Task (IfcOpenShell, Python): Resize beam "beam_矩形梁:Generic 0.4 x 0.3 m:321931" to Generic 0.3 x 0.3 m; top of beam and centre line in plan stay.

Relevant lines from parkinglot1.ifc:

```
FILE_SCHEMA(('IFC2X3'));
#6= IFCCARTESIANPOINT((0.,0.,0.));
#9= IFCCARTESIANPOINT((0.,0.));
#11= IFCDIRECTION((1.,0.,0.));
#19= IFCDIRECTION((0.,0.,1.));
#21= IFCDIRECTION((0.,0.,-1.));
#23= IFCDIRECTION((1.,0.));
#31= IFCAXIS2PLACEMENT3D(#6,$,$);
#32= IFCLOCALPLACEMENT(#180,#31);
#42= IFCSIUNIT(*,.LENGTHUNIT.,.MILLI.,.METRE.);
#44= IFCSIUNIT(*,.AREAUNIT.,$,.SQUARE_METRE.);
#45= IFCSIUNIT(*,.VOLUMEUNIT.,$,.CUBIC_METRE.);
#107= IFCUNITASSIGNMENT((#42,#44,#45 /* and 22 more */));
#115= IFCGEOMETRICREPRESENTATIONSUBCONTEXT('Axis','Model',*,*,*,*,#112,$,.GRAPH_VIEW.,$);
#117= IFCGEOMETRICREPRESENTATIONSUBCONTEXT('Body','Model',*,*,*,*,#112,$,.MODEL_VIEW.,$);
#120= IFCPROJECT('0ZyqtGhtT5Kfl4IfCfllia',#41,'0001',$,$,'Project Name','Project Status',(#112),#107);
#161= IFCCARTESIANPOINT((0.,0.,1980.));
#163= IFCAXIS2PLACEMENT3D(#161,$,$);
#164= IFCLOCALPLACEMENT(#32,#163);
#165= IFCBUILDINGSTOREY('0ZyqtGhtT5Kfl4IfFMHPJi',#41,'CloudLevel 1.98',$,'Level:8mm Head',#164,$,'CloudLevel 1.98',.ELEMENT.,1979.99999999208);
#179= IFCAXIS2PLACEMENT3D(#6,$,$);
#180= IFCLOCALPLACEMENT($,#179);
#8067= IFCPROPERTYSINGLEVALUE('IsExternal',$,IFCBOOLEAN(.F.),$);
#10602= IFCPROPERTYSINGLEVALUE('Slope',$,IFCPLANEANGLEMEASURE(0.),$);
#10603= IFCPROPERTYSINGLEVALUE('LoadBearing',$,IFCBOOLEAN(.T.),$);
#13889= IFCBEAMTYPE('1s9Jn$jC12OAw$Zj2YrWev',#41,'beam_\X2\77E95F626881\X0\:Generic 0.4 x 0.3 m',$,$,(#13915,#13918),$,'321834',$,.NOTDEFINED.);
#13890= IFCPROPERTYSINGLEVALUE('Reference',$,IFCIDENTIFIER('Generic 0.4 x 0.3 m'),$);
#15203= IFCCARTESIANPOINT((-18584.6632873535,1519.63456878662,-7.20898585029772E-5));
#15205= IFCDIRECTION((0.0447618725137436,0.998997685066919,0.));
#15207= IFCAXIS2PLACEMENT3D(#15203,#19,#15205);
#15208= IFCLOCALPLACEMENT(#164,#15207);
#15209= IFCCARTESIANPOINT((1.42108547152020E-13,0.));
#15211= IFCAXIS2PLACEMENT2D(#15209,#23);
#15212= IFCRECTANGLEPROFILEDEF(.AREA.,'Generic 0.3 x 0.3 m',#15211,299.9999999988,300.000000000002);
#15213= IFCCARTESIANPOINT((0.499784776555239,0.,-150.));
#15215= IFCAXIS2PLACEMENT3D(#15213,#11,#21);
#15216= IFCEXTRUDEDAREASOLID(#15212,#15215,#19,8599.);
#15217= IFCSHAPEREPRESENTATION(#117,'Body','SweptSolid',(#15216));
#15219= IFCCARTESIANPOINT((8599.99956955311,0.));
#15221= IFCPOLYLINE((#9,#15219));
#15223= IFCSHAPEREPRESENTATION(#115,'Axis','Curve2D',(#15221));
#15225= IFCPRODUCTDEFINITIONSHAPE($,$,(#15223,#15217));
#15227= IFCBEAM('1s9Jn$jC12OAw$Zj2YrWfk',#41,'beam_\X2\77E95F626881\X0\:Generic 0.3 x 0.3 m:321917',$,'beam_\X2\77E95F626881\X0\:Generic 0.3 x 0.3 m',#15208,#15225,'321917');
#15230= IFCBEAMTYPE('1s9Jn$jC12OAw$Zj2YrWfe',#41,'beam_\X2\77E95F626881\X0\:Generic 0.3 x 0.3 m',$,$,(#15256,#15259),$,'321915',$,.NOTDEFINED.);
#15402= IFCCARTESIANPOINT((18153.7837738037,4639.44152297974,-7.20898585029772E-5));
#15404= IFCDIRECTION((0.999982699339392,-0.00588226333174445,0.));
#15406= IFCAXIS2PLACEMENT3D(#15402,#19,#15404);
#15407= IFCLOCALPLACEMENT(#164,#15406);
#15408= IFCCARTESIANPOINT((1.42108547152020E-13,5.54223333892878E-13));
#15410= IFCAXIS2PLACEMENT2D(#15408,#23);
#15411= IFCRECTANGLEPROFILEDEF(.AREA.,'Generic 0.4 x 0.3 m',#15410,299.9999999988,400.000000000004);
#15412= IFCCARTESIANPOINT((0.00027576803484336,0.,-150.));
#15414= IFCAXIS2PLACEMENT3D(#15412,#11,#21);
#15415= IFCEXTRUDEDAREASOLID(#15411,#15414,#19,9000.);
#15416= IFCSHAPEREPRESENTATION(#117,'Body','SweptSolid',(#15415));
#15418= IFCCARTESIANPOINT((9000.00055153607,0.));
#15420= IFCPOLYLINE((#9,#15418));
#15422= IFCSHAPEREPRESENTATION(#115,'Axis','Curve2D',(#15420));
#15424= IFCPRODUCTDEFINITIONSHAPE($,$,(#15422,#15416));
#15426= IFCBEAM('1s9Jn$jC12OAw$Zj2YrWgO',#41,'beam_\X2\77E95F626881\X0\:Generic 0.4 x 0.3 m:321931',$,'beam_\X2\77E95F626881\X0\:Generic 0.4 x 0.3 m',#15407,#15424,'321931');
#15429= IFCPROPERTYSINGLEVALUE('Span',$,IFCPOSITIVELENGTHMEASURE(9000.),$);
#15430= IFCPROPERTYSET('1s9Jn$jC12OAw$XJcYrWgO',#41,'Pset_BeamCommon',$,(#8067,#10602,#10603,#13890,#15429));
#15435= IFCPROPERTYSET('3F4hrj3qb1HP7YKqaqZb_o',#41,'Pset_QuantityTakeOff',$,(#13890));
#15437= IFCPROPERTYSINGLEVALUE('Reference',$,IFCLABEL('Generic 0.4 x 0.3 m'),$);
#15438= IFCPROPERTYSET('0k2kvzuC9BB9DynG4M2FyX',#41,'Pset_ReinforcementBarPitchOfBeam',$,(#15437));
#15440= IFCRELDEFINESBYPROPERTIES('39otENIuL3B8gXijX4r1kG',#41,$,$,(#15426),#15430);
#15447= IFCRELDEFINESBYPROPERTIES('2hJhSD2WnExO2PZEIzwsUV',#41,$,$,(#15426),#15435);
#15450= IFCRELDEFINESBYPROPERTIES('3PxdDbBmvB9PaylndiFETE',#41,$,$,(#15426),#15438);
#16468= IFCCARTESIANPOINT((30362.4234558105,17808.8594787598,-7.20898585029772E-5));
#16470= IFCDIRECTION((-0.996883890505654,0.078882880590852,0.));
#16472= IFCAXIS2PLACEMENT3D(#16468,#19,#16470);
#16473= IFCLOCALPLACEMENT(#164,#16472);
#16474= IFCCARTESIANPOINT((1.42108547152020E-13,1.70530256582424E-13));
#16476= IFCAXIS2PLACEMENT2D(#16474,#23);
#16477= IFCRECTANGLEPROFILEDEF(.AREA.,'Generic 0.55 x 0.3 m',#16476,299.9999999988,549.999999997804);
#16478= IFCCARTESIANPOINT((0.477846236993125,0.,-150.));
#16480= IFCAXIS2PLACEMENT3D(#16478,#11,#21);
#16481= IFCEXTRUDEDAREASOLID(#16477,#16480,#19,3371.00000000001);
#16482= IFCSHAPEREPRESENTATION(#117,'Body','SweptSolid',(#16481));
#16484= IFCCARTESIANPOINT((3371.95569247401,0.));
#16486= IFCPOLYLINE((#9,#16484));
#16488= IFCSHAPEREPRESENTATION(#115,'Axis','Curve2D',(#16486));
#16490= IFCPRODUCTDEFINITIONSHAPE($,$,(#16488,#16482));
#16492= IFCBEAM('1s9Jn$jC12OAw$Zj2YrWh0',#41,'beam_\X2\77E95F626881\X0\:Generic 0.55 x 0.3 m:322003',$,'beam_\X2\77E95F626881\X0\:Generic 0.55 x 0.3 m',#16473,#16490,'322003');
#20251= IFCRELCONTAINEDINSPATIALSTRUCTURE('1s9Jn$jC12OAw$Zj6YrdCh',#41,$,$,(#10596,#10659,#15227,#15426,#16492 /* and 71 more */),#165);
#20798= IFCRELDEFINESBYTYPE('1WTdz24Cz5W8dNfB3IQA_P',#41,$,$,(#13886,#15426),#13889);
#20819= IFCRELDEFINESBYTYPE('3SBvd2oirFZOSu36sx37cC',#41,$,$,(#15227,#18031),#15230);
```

```python
import ifcopenshell
import ifcopenshell.api.pset
import ifcopenshell.api.type
import ifcopenshell.util.element
import ifcopenshell.util.representation

model = ifcopenshell.open("parkinglot1.ifc")

member = model.by_guid("1s9Jn$jC12OAw$Zj2YrWgO")
source = next(p for p in model.by_type("IfcRectangleProfileDef") if p.ProfileName == "Generic 0.3 x 0.3 m")

body = ifcopenshell.util.representation.get_representation(member, "Model", "Body")
solid = body.Items[0]
old_profile = solid.SweptArea

# Copy the section's sizes but keep this member's own profile position.
profile = ifcopenshell.util.element.copy(model, source)
# Profiles are centred, so shift by half the change in depth to hold the top.
shift = (old_profile.XDim - profile.XDim) / 2
x, y = old_profile.Position.Location.Coordinates
up = (-1.0, 0.0)  # upwards, in the solid's own plane
location = model.createIfcCartesianPoint((x + up[0] * shift, y + up[1] * shift))
profile.Position = model.createIfcAxis2Placement2D(location, old_profile.Position.RefDirection)
solid.SweptArea = profile
if not model.get_total_inverses(old_profile):
    ifcopenshell.util.element.remove_deep2(model, old_profile)

new_type = model.by_id(15230)
ifcopenshell.api.type.assign_type(
    model, related_objects=[member], relating_type=new_type, should_map_representations=False
)
member.Name = member.Name.replace("Generic 0.4 x 0.3 m", "Generic 0.3 x 0.3 m")
member.ObjectType = "beam_矩形梁:Generic 0.3 x 0.3 m"
pset = model.by_id(ifcopenshell.util.element.get_pset(member, "Pset_BeamCommon", should_inherit=False)["id"])
ifcopenshell.api.pset.edit_pset(model, pset=pset, properties={"Reference": "Generic 0.3 x 0.3 m"})
pset = model.by_id(ifcopenshell.util.element.get_pset(member, "Pset_QuantityTakeOff", should_inherit=False)["id"])
ifcopenshell.api.pset.edit_pset(model, pset=pset, properties={"Reference": "Generic 0.3 x 0.3 m"})
pset = model.by_id(ifcopenshell.util.element.get_pset(member, "Pset_ReinforcementBarPitchOfBeam", should_inherit=False)["id"])
ifcopenshell.api.pset.edit_pset(model, pset=pset, properties={"Reference": "Generic 0.3 x 0.3 m"})

print(solid.SweptArea)

model.write("parkinglot1-out.ifc")
```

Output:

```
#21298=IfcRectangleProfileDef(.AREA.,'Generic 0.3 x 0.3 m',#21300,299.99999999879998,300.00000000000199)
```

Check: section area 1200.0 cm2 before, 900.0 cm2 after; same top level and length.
